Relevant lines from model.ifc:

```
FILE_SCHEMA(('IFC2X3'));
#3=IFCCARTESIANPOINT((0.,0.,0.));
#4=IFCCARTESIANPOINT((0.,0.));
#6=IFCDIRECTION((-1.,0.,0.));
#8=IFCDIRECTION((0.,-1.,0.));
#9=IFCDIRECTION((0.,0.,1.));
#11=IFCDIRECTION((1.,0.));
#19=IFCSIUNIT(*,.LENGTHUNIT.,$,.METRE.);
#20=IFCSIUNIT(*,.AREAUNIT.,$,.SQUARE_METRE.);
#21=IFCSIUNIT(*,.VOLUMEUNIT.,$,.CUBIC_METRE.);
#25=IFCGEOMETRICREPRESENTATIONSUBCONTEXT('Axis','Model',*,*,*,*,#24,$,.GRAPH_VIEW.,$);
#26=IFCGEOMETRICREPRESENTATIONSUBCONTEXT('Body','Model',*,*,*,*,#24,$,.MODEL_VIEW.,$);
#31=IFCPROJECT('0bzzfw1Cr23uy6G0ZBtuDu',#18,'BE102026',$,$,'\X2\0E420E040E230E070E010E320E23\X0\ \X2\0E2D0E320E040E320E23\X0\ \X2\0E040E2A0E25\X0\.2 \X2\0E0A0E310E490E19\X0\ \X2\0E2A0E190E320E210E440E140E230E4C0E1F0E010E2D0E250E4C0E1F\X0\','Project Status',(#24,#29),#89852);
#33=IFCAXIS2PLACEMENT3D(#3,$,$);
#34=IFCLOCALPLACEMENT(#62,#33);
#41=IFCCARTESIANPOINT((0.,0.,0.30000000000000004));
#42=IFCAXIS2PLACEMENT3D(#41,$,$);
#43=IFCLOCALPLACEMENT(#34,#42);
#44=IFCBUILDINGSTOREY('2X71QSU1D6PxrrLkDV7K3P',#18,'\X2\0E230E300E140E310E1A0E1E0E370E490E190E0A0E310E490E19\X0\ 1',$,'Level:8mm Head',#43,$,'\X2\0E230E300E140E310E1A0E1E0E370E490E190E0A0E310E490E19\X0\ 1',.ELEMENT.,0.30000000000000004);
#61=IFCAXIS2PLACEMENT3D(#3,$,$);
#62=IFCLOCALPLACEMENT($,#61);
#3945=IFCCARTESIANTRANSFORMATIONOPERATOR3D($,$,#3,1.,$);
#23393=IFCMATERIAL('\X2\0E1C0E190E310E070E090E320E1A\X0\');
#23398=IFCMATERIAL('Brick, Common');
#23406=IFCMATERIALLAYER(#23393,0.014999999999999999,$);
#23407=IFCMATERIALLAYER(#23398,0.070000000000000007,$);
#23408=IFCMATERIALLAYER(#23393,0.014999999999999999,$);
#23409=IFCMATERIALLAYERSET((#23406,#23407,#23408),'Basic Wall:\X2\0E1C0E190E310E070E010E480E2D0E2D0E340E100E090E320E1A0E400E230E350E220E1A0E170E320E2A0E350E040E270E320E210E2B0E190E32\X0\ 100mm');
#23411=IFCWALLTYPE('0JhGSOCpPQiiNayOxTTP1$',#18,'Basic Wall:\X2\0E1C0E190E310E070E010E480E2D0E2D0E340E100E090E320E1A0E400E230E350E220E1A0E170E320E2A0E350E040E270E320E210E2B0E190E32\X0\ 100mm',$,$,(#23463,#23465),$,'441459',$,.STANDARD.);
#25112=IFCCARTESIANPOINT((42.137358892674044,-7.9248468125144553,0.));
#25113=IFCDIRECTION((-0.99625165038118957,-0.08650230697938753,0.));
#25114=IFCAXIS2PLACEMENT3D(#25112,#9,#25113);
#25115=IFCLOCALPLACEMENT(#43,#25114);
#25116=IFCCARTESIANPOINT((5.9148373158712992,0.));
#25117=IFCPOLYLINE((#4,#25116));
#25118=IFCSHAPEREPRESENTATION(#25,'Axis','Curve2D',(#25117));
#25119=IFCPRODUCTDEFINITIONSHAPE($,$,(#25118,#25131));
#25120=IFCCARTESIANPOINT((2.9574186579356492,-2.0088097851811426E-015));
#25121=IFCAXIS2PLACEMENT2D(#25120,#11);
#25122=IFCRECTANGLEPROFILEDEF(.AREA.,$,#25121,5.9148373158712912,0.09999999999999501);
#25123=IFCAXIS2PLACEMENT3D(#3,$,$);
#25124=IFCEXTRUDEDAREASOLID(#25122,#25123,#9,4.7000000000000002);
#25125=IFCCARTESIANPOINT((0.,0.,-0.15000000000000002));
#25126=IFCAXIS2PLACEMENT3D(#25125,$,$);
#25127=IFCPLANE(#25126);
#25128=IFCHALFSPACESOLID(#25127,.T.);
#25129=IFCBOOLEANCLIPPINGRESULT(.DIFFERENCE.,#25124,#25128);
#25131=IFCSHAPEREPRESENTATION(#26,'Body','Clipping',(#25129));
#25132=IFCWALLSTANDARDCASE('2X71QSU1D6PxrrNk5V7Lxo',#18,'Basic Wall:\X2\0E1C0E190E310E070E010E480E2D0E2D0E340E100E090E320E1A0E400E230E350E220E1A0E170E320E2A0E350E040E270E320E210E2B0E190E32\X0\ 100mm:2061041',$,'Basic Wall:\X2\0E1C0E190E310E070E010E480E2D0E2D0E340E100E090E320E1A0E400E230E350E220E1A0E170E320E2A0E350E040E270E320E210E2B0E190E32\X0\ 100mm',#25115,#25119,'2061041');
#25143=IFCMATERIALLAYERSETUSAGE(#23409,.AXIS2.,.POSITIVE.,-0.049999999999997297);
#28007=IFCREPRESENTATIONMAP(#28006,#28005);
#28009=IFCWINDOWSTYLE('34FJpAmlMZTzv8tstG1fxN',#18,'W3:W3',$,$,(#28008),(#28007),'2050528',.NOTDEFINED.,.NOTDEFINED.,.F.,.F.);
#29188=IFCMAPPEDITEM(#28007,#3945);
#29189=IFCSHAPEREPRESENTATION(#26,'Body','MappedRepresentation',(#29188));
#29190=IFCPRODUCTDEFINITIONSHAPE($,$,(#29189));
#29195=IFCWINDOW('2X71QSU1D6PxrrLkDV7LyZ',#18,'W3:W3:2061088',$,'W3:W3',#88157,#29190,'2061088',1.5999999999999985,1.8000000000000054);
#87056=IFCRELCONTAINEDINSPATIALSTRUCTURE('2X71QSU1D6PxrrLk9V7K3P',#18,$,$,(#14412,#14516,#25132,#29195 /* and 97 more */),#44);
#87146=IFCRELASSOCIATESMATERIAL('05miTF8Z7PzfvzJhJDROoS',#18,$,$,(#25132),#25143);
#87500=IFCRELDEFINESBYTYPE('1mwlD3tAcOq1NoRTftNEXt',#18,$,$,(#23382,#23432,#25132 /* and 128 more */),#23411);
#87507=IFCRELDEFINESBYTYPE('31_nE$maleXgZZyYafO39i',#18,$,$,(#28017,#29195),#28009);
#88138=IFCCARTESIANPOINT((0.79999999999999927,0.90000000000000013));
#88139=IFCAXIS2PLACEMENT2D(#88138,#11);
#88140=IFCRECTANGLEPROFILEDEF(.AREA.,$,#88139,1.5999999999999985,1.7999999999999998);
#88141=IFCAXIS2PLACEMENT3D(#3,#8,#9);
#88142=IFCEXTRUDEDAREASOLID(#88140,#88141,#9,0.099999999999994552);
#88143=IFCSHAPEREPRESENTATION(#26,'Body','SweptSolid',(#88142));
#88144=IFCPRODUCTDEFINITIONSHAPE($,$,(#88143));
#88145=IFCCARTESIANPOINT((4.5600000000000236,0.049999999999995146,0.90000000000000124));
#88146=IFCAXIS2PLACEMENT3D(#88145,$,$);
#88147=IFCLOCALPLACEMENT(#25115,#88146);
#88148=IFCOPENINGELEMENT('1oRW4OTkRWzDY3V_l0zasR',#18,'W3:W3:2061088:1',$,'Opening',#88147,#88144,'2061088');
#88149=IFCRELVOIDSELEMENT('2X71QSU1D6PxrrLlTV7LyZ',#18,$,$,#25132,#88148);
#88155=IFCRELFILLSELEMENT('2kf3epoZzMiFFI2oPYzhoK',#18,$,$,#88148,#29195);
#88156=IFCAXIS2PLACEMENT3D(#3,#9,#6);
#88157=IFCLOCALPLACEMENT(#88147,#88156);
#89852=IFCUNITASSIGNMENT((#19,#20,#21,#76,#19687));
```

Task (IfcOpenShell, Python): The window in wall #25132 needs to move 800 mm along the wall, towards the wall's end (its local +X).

```python
import ifcopenshell
import ifcopenshell.api.geometry
import ifcopenshell.util.placement

model = ifcopenshell.open("model.ifc")

window = model.by_guid("2X71QSU1D6PxrrLkDV7LyZ")
opening = window.FillsVoids[0].RelatingOpeningElement
wall = opening.VoidsElements[0].RelatingBuildingElement

wall_matrix = ifcopenshell.util.placement.get_local_placement(wall.ObjectPlacement)
shift = wall_matrix[:3, 0] * 0.8
before = ifcopenshell.util.placement.get_local_placement(window.ObjectPlacement)[:3, 3].copy()

# The window is placed relative to its opening, so it follows when the opening moves.
matrix = ifcopenshell.util.placement.get_local_placement(opening.ObjectPlacement)
matrix[:3, 3] += shift
ifcopenshell.api.geometry.edit_object_placement(
    model, product=opening, matrix=matrix, is_si=False, should_transform_children=True
)

after = ifcopenshell.util.placement.get_local_placement(window.ObjectPlacement)[:3, 3]
print("window moved by", (after - before).round(3) + 0.0)

model.write("model_edited.ifc")
```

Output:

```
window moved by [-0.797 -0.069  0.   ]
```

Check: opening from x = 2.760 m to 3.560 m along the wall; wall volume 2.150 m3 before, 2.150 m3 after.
